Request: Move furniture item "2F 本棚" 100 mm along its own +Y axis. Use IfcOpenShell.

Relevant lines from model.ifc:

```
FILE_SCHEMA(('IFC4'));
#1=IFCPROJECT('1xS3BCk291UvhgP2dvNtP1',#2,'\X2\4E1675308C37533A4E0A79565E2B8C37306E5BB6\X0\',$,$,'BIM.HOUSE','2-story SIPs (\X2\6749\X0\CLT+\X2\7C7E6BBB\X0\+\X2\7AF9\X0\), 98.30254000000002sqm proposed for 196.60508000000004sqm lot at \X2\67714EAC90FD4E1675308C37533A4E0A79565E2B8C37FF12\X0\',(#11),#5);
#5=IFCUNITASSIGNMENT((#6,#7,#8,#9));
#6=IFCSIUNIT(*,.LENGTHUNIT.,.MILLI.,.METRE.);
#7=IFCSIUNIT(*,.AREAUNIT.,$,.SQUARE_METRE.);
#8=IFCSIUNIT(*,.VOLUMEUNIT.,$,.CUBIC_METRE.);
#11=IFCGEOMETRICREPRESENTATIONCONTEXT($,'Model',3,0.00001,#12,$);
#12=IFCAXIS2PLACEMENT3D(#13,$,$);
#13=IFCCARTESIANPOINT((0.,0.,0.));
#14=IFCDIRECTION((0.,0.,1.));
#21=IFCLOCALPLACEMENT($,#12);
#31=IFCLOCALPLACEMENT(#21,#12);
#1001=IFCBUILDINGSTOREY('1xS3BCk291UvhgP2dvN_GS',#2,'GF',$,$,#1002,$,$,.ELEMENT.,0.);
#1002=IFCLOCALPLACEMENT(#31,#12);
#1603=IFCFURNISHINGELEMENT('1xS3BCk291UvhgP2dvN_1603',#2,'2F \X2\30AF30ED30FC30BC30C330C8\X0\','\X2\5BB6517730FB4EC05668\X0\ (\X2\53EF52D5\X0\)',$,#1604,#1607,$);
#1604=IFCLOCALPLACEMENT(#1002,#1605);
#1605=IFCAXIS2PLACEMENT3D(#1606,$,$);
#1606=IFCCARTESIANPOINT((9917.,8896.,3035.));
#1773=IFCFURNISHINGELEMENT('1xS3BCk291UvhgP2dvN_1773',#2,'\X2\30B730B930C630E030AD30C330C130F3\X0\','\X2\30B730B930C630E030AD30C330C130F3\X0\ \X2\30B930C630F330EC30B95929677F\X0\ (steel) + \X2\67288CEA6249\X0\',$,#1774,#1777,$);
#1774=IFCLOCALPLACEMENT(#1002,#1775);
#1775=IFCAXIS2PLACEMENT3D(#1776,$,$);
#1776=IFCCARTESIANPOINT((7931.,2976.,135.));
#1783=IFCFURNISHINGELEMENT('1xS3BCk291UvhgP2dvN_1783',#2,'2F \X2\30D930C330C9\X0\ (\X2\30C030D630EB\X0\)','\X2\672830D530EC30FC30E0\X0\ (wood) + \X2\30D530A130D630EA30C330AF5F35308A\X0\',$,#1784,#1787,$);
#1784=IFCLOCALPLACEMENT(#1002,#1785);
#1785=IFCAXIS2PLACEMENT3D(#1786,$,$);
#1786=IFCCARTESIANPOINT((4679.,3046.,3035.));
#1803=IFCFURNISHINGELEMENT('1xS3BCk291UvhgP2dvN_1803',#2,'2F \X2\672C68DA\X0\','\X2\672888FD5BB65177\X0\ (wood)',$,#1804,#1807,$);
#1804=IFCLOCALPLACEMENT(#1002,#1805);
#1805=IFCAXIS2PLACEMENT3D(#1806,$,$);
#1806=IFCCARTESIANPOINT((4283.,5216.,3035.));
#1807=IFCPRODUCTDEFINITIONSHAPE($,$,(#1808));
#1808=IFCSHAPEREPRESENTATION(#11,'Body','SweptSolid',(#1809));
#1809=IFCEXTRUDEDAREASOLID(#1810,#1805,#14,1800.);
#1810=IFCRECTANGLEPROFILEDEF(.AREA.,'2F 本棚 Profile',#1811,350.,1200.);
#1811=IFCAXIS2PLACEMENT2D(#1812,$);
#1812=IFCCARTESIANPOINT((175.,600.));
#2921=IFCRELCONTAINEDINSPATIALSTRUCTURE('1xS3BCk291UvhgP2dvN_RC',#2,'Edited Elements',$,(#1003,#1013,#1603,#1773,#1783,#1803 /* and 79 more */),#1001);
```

```python
import ifcopenshell
import ifcopenshell.api.geometry
import ifcopenshell.util.placement

model = ifcopenshell.open("model.ifc")

item = model.by_guid("1xS3BCk291UvhgP2dvN_1803")
matrix = ifcopenshell.util.placement.get_local_placement(item.ObjectPlacement)
matrix[:3, 3] += matrix[:3, 1] * 100.0
ifcopenshell.api.geometry.edit_object_placement(model, product=item, matrix=matrix, is_si=False)

print(ifcopenshell.util.placement.get_local_placement(item.ObjectPlacement).round(3) + 0.0)

model.write("model_updated.ifc")
```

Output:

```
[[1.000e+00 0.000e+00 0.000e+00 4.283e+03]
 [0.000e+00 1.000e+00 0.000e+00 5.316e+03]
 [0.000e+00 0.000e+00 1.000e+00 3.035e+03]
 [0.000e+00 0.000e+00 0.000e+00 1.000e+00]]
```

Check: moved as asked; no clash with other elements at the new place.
